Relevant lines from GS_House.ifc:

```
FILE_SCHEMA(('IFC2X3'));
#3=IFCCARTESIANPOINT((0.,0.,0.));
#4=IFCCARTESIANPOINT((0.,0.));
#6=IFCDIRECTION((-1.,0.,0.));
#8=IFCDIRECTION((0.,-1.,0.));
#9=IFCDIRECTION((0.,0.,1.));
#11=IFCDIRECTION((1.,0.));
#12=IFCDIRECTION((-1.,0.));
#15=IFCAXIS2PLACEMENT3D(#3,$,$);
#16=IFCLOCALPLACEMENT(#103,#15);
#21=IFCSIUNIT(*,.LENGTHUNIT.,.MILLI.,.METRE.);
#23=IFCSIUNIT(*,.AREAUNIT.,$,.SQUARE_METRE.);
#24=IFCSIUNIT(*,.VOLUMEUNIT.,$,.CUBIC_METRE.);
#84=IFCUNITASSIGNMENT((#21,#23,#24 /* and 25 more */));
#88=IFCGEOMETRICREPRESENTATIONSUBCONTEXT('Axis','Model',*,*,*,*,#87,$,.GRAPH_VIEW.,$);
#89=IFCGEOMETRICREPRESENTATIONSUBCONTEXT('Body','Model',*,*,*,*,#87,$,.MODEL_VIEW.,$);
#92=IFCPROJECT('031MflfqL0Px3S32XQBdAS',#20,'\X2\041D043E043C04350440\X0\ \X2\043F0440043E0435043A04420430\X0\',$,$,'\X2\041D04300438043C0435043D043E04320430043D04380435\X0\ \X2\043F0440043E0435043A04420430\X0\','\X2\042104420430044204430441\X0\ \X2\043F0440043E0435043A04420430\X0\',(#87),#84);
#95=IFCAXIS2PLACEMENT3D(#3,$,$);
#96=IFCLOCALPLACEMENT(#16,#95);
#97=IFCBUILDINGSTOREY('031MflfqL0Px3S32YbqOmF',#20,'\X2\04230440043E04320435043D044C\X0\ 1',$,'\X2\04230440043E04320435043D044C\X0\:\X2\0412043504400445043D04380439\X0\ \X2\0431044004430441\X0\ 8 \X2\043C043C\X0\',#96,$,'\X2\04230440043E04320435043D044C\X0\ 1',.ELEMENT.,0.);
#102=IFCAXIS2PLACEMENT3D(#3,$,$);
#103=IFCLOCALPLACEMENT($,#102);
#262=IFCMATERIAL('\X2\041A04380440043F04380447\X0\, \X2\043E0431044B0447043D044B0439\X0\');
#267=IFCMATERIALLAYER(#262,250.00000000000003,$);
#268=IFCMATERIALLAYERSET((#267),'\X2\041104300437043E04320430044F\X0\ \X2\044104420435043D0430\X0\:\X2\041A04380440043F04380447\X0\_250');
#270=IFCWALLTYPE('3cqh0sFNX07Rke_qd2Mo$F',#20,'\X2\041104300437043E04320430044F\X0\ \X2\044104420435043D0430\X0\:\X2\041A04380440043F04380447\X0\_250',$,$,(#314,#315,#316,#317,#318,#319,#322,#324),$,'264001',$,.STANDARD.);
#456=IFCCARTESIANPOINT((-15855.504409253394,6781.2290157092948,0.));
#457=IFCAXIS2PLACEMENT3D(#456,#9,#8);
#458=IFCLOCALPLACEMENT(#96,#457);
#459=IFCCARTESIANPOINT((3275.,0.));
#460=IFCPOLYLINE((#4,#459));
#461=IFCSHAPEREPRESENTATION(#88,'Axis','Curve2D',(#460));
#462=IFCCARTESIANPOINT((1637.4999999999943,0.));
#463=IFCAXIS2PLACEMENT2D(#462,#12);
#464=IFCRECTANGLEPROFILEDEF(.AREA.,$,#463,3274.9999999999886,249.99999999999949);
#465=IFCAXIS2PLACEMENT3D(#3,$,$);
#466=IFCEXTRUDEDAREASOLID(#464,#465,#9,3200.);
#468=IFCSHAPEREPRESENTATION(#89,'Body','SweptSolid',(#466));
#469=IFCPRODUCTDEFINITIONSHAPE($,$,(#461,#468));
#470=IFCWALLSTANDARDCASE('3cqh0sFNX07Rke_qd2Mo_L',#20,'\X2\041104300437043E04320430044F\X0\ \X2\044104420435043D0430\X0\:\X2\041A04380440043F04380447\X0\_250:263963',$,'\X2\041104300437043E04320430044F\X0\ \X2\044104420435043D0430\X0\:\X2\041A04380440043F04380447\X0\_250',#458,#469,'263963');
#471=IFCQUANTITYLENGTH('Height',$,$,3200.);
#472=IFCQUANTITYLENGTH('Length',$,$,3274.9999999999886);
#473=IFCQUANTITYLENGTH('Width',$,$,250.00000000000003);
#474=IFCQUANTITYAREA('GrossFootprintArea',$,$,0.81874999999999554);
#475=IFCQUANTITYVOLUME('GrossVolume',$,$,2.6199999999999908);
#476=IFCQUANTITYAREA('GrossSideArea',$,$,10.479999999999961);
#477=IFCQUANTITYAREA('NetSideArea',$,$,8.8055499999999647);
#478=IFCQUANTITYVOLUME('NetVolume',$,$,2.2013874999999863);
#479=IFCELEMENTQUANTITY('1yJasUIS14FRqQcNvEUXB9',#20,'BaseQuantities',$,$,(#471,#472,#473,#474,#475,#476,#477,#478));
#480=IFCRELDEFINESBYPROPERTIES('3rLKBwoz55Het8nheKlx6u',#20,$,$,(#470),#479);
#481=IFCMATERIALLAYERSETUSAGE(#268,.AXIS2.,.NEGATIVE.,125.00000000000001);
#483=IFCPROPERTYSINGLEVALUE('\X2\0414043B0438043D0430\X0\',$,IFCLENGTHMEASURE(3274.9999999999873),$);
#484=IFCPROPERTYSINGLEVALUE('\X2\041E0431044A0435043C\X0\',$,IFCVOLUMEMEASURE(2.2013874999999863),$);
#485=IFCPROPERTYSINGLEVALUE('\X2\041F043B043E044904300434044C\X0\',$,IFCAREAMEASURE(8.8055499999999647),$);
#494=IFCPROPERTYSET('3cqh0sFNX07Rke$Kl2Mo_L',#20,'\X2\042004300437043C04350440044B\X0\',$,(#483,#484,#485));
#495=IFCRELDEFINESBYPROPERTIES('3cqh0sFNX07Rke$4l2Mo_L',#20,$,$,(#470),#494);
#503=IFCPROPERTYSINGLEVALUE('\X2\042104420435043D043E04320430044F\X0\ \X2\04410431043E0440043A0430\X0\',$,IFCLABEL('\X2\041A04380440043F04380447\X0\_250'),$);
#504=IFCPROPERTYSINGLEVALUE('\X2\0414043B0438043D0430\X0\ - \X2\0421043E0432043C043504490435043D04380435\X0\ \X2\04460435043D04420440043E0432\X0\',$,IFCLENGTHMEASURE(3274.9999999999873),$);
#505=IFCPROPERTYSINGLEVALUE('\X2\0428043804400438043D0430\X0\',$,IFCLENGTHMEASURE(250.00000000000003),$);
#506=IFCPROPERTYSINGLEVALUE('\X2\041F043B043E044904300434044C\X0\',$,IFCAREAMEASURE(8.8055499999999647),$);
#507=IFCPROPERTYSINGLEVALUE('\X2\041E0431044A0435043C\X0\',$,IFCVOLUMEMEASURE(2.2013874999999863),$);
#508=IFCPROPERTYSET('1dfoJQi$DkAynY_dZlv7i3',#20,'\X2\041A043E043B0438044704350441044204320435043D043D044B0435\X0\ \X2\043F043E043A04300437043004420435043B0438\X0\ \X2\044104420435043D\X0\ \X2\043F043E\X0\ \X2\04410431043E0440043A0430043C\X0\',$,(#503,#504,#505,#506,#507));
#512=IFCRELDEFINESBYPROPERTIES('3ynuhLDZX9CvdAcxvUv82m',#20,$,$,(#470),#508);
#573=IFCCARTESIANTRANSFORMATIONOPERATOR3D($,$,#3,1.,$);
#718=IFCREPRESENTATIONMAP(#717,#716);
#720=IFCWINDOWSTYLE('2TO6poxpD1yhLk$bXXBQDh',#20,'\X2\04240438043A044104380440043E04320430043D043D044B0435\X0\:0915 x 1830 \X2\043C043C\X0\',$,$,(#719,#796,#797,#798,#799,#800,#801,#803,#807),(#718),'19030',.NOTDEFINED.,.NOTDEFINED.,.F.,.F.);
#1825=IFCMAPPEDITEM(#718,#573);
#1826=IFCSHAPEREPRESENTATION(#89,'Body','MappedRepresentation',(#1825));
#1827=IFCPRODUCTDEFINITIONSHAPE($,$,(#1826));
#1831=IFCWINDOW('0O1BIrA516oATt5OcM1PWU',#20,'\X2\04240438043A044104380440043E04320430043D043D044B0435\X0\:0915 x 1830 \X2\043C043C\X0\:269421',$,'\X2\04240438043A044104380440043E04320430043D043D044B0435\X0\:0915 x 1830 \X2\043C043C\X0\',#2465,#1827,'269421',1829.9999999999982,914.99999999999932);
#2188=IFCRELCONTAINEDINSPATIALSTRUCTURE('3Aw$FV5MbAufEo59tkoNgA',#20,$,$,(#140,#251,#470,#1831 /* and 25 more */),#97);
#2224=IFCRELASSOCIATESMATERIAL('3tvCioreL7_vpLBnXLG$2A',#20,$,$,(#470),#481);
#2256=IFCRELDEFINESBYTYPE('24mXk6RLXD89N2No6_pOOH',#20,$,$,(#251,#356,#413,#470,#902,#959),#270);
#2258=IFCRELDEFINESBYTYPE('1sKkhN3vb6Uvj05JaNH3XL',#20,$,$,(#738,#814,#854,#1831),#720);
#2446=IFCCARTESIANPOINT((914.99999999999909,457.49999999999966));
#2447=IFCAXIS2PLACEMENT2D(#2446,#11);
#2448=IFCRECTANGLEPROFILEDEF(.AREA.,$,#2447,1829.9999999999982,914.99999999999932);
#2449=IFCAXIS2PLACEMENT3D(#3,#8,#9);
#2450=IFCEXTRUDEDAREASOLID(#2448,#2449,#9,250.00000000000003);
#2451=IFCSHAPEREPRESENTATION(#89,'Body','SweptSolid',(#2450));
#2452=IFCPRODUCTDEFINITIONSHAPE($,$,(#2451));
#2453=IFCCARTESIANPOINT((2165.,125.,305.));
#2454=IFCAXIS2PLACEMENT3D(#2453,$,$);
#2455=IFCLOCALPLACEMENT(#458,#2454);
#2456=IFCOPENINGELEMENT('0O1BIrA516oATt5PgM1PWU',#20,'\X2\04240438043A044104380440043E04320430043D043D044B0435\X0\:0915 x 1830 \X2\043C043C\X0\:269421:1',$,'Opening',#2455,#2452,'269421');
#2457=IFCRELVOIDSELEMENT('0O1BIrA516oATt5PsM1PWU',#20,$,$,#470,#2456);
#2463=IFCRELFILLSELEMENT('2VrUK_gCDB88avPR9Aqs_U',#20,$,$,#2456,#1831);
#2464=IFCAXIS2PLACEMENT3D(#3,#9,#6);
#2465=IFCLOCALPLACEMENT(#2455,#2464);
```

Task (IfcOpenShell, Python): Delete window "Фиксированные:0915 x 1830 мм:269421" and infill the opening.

```python
import ifcopenshell
import ifcopenshell.api.feature
import ifcopenshell.api.pset
import ifcopenshell.api.root
import ifcopenshell.geom
import ifcopenshell.util.element
import ifcopenshell.util.shape
import ifcopenshell.util.unit

model = ifcopenshell.open("GS_House.ifc")
area_scale = ifcopenshell.util.unit.calculate_unit_scale(model, "AREAUNIT")
volume_scale = ifcopenshell.util.unit.calculate_unit_scale(model, "VOLUMEUNIT")
settings = ifcopenshell.geom.settings()


def volume(element):
    """Net volume in cubic metres, openings subtracted."""
    shape = ifcopenshell.geom.create_shape(settings, element)
    return ifcopenshell.util.shape.get_volume(shape.geometry)


window = model.by_guid("0O1BIrA516oATt5OcM1PWU")
opening = window.FillsVoids[0].RelatingOpeningElement
wall = opening.VoidsElements[0].RelatingBuildingElement
before = volume(wall)

ifcopenshell.api.root.remove_product(model, product=window)
ifcopenshell.api.feature.remove_feature(model, feature=opening)

after = volume(wall)
thickness = 0.25  # wall thickness in metres

# Update the wall's stored quantities.
qto = model.by_id(ifcopenshell.util.element.get_pset(wall, "BaseQuantities", should_inherit=False)["id"])
ifcopenshell.api.pset.edit_qto(model, qto=qto, properties={
    "NetSideArea": after / thickness / area_scale,
    "NetVolume": after / volume_scale,
})
pset = model.by_id(ifcopenshell.util.element.get_pset(wall, "Размеры", should_inherit=False)["id"])
ifcopenshell.api.pset.edit_pset(model, pset=pset, properties={
    "Объем": model.create_entity("IfcVolumeMeasure", after / volume_scale),
    "Площадь": model.create_entity("IfcAreaMeasure", after / thickness / area_scale),
})
pset = model.by_id(ifcopenshell.util.element.get_pset(wall, "Количественные показатели стен по сборкам", should_inherit=False)["id"])
ifcopenshell.api.pset.edit_pset(model, pset=pset, properties={
    "Площадь": model.create_entity("IfcAreaMeasure", after / thickness / area_scale),
    "Объем": model.create_entity("IfcVolumeMeasure", after / volume_scale),
})

print(f"wall volume {before:.3f} -> {after:.3f} m3")

model.write("GS_House_edited.ifc")
```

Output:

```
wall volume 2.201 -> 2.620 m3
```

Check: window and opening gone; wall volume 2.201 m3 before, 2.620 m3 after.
